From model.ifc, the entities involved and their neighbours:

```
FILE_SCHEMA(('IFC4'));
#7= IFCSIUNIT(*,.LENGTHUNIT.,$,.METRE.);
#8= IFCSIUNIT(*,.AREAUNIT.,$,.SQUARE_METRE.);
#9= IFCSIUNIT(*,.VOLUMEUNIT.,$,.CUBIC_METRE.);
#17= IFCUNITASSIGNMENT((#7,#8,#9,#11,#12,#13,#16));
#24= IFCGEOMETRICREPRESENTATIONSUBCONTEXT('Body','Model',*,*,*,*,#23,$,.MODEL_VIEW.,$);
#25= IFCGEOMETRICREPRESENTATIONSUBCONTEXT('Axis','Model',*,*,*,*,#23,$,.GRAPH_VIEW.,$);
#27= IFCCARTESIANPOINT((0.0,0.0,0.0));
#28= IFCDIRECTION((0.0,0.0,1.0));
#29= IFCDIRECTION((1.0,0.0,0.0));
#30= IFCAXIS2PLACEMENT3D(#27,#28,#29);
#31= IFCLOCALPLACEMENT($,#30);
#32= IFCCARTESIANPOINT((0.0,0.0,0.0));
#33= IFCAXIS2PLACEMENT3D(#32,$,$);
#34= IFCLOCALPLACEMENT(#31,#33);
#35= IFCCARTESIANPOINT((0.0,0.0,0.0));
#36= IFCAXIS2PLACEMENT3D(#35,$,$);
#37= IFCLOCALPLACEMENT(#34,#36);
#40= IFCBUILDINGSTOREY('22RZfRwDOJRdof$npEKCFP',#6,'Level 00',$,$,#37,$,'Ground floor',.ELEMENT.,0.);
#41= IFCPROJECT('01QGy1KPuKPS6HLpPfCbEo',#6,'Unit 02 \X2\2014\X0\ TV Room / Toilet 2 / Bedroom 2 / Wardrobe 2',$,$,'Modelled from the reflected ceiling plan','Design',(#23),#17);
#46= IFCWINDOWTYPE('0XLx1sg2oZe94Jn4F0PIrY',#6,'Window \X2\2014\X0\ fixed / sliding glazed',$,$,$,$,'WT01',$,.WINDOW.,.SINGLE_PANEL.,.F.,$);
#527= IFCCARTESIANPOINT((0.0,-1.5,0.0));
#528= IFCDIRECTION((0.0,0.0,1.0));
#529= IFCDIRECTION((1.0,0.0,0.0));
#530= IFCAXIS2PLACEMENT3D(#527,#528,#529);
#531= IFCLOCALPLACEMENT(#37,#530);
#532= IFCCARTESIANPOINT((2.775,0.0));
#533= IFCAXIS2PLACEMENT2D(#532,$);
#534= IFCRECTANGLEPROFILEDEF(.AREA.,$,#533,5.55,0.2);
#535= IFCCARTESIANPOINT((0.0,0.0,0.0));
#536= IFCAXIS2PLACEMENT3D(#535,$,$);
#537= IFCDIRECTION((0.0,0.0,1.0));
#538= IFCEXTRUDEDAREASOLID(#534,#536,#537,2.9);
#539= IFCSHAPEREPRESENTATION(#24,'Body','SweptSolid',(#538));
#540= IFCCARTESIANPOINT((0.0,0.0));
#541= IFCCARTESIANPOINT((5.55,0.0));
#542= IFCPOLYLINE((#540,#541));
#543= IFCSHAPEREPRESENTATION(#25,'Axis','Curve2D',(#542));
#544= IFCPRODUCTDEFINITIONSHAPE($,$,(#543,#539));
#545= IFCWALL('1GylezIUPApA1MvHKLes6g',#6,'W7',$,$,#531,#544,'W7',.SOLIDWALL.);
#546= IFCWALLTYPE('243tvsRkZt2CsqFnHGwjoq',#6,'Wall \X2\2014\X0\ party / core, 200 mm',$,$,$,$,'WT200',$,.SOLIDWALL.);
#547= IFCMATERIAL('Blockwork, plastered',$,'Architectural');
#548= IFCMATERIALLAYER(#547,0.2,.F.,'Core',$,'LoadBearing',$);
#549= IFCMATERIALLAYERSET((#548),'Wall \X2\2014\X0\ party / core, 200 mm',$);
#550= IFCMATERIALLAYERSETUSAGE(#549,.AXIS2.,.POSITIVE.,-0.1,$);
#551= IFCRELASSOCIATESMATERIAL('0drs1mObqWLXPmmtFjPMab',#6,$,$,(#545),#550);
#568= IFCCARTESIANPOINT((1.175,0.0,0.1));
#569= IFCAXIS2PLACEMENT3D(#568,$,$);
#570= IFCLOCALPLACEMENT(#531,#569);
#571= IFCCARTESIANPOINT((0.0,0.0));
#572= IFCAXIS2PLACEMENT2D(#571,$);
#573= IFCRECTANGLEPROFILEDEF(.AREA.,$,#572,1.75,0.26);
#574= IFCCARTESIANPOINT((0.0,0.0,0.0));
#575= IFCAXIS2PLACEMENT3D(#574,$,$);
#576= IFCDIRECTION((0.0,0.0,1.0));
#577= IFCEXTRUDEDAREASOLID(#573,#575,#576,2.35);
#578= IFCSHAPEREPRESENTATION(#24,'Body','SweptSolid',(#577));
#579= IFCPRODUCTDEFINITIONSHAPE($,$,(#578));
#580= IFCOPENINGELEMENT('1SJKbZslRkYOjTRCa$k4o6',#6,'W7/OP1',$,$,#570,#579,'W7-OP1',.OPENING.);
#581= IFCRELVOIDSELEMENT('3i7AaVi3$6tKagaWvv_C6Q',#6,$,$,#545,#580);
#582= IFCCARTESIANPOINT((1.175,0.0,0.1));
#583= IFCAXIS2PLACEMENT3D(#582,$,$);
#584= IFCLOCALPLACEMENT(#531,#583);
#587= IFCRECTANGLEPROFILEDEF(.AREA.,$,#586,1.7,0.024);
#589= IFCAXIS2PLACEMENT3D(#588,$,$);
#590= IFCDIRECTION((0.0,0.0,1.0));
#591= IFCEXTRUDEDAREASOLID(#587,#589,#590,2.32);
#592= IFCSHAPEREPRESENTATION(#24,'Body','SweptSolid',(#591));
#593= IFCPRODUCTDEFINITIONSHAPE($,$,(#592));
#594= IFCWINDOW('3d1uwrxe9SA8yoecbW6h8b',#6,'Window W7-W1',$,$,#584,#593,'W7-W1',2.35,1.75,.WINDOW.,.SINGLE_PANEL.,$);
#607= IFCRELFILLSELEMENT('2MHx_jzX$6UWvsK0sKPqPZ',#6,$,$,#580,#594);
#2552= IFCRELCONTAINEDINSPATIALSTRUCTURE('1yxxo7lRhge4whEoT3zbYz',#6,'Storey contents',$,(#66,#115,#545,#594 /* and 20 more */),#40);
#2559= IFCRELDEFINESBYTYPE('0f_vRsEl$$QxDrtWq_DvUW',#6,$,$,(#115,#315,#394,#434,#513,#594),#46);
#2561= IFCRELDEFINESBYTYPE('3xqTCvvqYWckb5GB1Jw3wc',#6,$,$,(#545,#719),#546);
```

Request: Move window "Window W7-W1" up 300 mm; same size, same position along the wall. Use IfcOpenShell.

```python
import numpy as np
import ifcopenshell
import ifcopenshell.api.geometry
import ifcopenshell.util.placement
import ifcopenshell.util.unit

model = ifcopenshell.open("model.ifc")
unit_scale = ifcopenshell.util.unit.calculate_unit_scale(model)

window = model.by_guid("3d1uwrxe9SA8yoecbW6h8b")
opening = window.FillsVoids[0].RelatingOpeningElement
dz = 0.3 / unit_scale

shift = np.array([0.0, 0.0, dz])
# The window is not placed relative to its opening, so move both.
for product in (opening, window):
    matrix = ifcopenshell.util.placement.get_local_placement(product.ObjectPlacement)
    matrix[:3, 3] += shift
    ifcopenshell.api.geometry.edit_object_placement(model, product=product, matrix=matrix, is_si=False)

print(f"moved by {dz * unit_scale:+.3f} m")

model.write("model_v2.ifc")
```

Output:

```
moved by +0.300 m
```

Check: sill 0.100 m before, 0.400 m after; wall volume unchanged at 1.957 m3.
